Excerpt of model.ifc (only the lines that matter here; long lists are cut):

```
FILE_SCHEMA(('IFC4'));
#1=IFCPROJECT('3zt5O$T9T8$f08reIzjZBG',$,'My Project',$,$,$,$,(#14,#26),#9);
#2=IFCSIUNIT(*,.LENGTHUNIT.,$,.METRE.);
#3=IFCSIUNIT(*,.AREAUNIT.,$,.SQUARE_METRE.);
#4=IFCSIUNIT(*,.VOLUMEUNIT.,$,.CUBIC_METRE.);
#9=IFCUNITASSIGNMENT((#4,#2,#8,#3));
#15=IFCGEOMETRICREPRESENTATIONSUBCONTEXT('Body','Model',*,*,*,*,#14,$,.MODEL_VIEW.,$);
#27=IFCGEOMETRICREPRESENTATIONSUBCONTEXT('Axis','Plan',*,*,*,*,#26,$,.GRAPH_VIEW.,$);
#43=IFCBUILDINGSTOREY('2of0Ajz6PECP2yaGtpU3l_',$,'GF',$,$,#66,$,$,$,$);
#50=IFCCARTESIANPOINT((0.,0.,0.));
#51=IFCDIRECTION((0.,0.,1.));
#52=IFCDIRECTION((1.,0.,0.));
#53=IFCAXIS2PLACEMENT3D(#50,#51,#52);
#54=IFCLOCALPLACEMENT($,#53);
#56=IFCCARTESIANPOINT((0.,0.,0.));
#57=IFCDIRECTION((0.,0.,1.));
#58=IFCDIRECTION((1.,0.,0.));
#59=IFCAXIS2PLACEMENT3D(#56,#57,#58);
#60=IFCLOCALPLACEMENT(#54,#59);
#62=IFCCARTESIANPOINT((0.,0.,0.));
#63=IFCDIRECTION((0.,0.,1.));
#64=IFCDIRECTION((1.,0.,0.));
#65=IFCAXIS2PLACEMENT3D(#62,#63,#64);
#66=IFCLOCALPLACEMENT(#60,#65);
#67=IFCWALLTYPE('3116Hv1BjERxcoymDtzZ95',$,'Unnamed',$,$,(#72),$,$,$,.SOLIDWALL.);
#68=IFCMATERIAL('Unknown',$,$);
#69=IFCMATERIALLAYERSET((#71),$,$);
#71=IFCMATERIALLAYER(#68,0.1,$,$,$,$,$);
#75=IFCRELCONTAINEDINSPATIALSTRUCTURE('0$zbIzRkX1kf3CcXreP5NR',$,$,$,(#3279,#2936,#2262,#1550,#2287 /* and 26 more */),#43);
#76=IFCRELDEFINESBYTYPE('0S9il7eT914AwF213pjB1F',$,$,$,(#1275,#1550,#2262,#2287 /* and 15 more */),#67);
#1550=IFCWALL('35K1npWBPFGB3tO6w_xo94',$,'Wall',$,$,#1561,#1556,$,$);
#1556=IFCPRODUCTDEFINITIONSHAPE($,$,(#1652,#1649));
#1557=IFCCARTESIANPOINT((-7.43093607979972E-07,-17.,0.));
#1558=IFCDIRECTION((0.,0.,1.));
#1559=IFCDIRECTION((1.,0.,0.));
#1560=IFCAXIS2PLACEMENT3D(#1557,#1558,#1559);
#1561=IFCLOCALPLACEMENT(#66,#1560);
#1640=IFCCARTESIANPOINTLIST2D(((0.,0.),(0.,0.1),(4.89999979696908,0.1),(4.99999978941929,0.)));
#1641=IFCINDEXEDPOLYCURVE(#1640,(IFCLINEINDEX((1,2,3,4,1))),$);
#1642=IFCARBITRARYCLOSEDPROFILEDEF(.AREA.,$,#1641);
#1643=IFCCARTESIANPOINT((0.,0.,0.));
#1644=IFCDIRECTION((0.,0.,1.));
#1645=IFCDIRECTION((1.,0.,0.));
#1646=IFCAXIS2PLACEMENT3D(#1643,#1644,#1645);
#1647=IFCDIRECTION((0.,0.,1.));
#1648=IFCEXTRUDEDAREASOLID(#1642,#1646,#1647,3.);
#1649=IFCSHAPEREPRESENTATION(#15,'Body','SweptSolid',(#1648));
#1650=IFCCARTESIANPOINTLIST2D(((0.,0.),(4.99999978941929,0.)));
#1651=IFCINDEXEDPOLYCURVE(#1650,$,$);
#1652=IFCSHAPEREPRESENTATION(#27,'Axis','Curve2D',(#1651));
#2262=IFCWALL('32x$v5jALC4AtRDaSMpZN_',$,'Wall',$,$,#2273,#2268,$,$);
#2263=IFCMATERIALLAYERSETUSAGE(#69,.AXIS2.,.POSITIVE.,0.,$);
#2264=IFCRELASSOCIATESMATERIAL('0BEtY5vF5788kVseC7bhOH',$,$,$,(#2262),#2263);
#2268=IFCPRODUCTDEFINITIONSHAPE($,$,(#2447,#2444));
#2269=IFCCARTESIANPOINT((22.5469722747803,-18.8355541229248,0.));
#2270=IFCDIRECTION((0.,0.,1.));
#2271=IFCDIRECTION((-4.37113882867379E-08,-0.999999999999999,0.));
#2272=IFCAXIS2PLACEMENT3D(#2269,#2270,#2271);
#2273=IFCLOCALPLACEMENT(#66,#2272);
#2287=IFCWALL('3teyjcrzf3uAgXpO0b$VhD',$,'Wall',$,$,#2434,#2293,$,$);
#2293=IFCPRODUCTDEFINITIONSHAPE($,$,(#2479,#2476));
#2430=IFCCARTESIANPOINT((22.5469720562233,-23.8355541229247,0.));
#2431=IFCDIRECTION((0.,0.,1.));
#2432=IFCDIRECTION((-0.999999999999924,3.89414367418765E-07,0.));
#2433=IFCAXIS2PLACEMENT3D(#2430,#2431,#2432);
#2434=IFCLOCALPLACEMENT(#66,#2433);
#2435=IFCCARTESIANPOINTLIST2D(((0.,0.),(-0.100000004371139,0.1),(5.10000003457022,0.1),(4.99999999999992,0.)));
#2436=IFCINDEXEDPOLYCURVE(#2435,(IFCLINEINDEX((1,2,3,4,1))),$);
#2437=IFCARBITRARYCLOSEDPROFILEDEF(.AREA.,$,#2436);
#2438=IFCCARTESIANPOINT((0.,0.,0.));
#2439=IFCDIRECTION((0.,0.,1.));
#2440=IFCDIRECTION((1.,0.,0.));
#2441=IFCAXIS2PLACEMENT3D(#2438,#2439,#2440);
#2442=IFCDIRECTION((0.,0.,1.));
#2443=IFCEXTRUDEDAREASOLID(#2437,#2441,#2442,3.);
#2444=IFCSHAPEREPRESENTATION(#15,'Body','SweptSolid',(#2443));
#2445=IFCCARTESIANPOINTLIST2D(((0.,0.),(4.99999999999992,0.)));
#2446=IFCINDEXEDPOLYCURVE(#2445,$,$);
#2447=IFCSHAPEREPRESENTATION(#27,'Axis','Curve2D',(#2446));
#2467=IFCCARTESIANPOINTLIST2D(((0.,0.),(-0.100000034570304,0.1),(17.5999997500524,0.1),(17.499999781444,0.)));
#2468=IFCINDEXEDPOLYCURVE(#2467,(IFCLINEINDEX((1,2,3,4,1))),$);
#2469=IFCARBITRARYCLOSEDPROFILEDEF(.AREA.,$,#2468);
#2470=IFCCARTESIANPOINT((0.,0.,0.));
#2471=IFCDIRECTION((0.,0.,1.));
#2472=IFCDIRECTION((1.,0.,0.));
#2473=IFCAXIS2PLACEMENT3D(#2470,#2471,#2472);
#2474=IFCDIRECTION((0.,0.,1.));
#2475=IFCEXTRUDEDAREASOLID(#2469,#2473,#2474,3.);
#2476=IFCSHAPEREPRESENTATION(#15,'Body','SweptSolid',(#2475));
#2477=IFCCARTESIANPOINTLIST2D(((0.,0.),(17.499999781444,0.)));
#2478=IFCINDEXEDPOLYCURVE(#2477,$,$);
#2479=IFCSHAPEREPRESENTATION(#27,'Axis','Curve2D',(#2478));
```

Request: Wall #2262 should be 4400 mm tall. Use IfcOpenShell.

```python
import ifcopenshell
import ifcopenshell.geom
import ifcopenshell.util.representation
import ifcopenshell.util.shape

model = ifcopenshell.open("model.ifc")
settings = ifcopenshell.geom.settings()


def volume(element):
    """Net volume in cubic metres, openings subtracted."""
    shape = ifcopenshell.geom.create_shape(settings, element)
    return ifcopenshell.util.shape.get_volume(shape.geometry)


wall = model.by_guid("32x$v5jALC4AtRDaSMpZN_")
before = volume(wall)

body = ifcopenshell.util.representation.get_representation(wall, "Model", "Body")
solid = body.Items[0]
old_height = solid.Depth
solid.Depth = 4.4
after = volume(wall)

print(f"height {old_height:g} -> {solid.Depth:g}, volume {before:.3f} -> {after:.3f} m3")

model.write("model_rev.ifc")
```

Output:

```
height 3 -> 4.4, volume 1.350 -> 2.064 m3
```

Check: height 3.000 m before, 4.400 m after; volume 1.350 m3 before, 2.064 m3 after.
